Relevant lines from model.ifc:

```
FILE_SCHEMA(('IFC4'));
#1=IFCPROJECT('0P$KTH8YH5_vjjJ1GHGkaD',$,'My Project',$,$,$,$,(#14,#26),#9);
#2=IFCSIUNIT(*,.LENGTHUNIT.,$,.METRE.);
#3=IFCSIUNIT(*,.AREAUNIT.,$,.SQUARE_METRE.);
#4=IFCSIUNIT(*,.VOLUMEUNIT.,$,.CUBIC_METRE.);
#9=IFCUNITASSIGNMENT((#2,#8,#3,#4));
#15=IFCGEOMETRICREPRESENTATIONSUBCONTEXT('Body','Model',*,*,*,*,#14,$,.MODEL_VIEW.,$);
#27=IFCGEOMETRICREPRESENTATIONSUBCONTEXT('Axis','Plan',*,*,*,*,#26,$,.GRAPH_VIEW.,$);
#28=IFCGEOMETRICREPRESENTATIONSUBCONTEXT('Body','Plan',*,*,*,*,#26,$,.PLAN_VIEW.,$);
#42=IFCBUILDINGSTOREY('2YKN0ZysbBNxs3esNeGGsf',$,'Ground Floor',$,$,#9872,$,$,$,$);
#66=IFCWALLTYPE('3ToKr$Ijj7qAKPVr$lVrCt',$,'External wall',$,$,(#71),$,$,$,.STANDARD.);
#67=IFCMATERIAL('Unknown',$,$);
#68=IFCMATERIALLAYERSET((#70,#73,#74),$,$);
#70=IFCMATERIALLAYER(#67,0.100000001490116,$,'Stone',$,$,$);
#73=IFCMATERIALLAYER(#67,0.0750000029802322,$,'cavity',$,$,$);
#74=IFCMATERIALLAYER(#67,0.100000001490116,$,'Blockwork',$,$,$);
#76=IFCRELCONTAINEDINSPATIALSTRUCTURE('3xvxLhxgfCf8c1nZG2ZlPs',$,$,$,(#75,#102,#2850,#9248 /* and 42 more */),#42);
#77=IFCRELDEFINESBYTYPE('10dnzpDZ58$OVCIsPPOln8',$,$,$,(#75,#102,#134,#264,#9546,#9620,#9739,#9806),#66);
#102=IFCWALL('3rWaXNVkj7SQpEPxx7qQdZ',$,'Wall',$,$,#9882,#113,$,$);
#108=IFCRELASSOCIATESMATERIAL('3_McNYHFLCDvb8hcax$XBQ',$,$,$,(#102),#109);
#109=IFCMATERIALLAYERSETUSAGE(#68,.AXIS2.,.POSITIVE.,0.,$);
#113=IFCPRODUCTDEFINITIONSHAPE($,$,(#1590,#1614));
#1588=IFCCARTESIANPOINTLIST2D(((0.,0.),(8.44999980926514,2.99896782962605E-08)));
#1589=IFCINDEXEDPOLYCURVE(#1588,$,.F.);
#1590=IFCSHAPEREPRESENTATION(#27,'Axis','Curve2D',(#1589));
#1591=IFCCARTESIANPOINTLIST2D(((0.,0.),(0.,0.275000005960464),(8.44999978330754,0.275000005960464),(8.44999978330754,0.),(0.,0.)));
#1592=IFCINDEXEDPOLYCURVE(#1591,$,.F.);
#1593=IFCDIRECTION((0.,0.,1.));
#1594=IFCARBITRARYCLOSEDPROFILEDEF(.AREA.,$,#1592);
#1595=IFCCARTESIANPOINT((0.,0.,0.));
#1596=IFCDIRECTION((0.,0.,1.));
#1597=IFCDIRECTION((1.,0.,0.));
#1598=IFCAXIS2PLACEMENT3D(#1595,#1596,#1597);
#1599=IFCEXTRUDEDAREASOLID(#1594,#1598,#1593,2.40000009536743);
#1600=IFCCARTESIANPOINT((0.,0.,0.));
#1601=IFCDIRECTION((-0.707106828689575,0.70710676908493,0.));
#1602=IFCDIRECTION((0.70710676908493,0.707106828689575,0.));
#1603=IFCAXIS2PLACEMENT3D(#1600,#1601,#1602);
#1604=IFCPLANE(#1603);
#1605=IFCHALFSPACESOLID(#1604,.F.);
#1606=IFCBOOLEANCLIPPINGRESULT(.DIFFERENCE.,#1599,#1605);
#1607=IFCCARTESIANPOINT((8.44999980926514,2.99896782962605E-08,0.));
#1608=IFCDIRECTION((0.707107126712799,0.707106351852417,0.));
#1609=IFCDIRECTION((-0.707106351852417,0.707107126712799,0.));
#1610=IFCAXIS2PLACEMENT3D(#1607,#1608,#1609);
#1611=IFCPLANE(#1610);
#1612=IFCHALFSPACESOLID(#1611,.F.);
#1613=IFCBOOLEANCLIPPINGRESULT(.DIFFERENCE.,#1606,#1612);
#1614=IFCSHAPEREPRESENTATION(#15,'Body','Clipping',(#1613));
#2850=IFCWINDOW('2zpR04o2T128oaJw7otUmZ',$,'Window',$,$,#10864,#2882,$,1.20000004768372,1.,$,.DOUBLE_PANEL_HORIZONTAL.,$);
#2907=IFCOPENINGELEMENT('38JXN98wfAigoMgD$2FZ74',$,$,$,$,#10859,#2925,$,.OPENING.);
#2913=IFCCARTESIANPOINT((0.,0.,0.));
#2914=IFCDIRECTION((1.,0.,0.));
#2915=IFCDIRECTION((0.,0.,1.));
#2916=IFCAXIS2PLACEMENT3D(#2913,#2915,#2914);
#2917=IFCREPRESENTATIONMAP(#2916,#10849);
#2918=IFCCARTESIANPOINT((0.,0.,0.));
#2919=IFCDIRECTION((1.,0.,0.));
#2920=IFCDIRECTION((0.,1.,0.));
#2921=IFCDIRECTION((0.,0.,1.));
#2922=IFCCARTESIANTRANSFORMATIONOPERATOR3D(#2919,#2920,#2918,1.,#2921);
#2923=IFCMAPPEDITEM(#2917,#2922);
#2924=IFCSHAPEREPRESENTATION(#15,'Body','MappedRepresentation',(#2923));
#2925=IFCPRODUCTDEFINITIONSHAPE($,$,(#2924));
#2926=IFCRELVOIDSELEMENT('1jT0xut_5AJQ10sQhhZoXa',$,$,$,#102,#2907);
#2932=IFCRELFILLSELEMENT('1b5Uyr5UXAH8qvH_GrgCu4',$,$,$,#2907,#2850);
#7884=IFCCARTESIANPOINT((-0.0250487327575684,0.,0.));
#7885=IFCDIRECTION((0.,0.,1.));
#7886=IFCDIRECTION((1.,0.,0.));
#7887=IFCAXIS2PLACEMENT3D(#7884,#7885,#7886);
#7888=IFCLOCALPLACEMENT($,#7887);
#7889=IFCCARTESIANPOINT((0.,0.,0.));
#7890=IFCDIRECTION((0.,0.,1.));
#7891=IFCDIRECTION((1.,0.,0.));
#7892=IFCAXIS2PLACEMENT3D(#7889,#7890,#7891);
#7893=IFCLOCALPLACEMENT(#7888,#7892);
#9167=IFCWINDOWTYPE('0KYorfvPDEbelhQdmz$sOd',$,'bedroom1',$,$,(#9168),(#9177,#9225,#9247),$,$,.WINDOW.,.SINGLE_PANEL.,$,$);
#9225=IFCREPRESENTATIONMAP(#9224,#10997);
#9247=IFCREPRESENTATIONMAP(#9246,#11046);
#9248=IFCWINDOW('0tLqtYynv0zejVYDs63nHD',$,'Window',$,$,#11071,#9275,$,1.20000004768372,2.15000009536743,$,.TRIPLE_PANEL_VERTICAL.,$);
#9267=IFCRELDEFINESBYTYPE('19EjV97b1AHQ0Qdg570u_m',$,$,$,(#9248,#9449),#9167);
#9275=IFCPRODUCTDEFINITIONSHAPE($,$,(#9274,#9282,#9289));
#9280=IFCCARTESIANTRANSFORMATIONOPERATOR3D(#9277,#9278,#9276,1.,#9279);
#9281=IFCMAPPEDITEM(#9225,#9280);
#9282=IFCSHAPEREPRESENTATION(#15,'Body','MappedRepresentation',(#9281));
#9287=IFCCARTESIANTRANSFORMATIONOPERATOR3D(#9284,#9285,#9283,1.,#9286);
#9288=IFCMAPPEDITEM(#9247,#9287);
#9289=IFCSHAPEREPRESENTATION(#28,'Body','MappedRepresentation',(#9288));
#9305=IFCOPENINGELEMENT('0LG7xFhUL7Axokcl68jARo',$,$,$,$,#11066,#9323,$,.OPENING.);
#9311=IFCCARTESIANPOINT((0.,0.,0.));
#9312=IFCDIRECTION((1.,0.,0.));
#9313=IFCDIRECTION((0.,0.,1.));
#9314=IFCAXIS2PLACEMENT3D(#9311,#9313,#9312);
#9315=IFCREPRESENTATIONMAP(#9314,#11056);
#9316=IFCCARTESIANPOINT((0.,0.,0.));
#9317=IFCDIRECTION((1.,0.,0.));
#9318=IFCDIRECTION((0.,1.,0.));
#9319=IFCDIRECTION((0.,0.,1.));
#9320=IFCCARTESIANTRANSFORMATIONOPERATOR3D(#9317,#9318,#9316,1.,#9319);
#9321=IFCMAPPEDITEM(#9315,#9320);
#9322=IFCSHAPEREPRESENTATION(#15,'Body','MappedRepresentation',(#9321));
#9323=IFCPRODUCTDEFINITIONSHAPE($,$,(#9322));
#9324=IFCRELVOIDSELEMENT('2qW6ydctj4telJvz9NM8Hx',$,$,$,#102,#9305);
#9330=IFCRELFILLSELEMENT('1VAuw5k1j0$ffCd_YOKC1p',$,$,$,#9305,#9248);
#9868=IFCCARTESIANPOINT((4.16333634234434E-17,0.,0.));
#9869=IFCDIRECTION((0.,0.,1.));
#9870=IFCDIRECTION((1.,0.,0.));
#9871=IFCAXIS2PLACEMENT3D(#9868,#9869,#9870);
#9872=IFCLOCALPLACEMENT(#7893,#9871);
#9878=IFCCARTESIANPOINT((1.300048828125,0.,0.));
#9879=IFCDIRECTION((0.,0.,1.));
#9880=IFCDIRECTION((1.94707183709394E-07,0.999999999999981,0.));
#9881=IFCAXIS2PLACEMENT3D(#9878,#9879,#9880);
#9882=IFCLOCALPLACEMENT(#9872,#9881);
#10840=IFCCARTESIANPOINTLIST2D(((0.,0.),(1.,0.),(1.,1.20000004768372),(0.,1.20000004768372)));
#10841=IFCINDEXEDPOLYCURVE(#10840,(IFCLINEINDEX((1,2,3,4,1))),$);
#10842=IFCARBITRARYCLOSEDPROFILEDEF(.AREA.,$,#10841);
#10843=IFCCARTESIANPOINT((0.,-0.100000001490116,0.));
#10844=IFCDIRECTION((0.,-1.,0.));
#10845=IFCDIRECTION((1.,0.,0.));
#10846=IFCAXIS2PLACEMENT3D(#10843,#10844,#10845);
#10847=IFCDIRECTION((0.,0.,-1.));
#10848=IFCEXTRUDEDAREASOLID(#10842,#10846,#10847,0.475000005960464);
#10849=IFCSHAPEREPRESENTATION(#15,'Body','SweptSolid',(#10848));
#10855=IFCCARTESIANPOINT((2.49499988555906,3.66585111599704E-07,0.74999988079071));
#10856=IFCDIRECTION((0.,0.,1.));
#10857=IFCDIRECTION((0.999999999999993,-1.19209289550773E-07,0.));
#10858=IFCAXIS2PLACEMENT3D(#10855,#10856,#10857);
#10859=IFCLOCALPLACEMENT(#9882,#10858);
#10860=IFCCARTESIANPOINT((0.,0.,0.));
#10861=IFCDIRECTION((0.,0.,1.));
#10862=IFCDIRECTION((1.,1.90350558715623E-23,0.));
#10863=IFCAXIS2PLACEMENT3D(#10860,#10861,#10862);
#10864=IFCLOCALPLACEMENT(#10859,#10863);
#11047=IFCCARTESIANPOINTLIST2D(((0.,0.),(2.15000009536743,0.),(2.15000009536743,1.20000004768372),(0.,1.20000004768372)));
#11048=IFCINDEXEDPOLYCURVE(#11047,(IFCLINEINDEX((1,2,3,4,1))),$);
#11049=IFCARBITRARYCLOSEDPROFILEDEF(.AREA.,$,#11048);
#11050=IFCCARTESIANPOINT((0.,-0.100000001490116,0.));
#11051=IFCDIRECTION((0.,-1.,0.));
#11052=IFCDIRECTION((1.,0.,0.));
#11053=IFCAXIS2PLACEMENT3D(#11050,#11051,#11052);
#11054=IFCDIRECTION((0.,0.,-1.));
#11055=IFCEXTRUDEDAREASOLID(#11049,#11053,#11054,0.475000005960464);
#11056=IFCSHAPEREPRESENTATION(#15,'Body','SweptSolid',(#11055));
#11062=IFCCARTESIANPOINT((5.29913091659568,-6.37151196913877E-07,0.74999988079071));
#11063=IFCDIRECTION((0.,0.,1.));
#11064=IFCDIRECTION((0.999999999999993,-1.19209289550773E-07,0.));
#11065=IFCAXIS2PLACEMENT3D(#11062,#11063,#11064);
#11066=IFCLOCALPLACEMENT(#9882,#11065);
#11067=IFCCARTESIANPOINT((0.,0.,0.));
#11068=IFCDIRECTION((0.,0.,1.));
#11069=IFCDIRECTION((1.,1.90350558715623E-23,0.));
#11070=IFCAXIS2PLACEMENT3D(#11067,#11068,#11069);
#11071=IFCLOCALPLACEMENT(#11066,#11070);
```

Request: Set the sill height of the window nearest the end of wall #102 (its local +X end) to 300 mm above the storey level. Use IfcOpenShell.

```python
import numpy as np
import ifcopenshell
import ifcopenshell.api.geometry
import ifcopenshell.geom
import ifcopenshell.util.element
import ifcopenshell.util.placement
import ifcopenshell.util.shape
import ifcopenshell.util.unit

model = ifcopenshell.open("model.ifc")
unit_scale = ifcopenshell.util.unit.calculate_unit_scale(model)

window = model.by_id(9248)
opening = window.FillsVoids[0].RelatingOpeningElement
storey = ifcopenshell.util.element.get_container(window, ifc_class="IfcBuildingStorey")
level = ifcopenshell.util.placement.get_local_placement(storey.ObjectPlacement)[2, 3]

# The opening's origin need not be at the sill, so measure its lowest point.
shape = ifcopenshell.geom.create_shape(ifcopenshell.geom.settings(), opening)
bottom = ifcopenshell.util.shape.get_shape_bottom_elevation(shape, shape.geometry) / unit_scale
dz = level + 0.3 - bottom

shift = np.array([0.0, 0.0, dz])
# The window is placed relative to its opening, so it follows when the opening moves.
matrix = ifcopenshell.util.placement.get_local_placement(opening.ObjectPlacement)
matrix[:3, 3] += shift
ifcopenshell.api.geometry.edit_object_placement(
    model, product=opening, matrix=matrix, is_si=False, should_transform_children=True
)

print(f"moved by {dz * unit_scale:+.3f} m")

model.write("model_v2.ifc")
```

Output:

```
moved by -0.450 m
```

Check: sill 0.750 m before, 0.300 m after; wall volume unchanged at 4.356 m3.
